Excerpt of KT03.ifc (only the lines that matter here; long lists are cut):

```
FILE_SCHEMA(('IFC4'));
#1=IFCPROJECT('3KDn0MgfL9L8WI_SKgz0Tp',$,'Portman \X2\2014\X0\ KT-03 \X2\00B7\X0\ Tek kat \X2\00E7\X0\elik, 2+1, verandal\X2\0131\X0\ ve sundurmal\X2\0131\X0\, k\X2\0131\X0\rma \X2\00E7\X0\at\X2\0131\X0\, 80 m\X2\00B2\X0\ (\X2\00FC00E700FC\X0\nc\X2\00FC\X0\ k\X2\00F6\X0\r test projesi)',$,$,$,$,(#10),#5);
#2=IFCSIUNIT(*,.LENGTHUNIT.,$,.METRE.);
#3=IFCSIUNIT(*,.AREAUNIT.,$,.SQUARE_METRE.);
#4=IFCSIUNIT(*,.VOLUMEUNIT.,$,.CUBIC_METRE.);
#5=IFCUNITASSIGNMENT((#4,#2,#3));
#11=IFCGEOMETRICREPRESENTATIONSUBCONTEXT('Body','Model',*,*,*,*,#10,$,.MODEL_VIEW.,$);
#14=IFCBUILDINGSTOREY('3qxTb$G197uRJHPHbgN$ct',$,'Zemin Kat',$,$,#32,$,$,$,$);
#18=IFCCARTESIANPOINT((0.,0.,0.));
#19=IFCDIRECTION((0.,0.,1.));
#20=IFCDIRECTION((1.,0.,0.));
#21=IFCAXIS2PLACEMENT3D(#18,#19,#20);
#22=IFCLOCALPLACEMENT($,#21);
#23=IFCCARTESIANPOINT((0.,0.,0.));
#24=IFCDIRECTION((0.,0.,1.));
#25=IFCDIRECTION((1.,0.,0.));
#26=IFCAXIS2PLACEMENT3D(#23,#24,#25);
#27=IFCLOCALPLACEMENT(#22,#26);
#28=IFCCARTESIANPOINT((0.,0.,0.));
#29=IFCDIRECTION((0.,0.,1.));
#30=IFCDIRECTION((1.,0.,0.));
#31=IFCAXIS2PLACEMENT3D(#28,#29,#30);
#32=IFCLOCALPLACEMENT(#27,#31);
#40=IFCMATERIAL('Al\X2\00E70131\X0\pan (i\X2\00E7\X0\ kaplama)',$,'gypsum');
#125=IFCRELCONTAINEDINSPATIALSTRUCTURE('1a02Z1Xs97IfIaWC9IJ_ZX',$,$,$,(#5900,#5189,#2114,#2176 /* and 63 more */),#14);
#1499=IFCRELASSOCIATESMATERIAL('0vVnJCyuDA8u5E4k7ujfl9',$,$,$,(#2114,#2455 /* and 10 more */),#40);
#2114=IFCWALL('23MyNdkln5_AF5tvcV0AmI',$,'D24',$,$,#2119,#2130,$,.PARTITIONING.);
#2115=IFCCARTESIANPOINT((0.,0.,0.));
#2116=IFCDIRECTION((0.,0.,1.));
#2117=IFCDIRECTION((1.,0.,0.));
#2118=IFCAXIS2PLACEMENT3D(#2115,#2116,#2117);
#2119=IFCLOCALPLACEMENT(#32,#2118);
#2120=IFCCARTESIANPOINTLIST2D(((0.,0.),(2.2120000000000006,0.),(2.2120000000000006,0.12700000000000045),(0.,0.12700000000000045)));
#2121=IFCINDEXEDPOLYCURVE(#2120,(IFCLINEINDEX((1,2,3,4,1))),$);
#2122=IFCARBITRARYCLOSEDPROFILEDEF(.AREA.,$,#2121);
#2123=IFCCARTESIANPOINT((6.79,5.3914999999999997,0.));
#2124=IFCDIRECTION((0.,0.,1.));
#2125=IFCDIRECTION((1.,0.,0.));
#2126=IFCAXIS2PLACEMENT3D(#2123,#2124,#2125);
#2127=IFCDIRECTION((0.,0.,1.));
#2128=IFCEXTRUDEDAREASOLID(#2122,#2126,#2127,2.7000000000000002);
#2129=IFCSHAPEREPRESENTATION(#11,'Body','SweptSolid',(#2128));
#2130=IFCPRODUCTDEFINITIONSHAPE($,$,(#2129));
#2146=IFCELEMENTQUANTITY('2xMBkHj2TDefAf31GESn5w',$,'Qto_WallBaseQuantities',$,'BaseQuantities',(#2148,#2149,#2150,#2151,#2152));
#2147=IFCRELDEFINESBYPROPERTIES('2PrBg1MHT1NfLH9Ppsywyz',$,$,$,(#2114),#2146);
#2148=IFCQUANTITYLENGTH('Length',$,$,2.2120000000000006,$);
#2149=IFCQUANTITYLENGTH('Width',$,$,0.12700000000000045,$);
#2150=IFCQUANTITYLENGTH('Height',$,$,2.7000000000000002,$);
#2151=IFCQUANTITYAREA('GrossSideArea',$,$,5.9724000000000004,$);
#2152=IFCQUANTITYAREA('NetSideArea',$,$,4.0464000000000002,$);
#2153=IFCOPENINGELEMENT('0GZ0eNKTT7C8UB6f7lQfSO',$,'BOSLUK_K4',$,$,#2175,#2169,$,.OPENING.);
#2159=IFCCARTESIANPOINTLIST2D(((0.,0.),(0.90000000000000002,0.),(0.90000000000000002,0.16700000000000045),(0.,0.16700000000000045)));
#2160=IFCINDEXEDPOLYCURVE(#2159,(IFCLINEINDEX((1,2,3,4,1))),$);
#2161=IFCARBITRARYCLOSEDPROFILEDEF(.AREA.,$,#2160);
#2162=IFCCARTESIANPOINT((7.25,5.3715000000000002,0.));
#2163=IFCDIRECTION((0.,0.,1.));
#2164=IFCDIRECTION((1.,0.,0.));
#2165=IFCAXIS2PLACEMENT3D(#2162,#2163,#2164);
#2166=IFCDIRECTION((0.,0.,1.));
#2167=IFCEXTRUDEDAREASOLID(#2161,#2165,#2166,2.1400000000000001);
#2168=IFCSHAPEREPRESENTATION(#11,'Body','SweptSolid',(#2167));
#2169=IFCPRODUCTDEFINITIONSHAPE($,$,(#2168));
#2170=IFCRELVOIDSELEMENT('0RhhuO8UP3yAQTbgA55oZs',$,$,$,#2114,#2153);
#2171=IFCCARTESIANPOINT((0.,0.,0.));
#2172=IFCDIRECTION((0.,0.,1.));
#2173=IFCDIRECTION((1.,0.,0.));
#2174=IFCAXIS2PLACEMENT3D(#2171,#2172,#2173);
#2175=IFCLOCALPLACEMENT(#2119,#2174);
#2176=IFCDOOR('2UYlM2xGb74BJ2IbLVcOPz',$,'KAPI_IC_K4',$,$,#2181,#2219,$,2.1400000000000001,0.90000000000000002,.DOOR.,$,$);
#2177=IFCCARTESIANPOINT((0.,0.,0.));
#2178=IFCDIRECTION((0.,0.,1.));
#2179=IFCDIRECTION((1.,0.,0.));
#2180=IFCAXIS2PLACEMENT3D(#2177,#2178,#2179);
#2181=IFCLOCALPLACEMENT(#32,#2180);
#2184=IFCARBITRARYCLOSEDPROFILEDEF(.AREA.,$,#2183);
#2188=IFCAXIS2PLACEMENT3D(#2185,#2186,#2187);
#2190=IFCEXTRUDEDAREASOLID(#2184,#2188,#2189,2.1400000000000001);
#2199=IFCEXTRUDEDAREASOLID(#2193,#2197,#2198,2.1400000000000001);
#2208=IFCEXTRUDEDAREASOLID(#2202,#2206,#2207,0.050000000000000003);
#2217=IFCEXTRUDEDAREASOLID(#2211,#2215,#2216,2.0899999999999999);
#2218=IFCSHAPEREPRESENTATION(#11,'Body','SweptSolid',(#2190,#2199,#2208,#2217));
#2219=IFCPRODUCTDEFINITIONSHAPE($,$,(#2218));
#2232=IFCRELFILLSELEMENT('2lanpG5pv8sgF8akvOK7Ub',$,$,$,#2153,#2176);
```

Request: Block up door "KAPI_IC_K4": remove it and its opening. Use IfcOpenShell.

```python
import ifcopenshell
import ifcopenshell.api.feature
import ifcopenshell.api.pset
import ifcopenshell.api.root
import ifcopenshell.geom
import ifcopenshell.util.element
import ifcopenshell.util.shape
import ifcopenshell.util.unit

model = ifcopenshell.open("KT03.ifc")
area_scale = ifcopenshell.util.unit.calculate_unit_scale(model, "AREAUNIT")
settings = ifcopenshell.geom.settings()


def volume(element):
    """Net volume in cubic metres, openings subtracted."""
    shape = ifcopenshell.geom.create_shape(settings, element)
    return ifcopenshell.util.shape.get_volume(shape.geometry)


door = model.by_guid("2UYlM2xGb74BJ2IbLVcOPz")
opening = door.FillsVoids[0].RelatingOpeningElement
wall = opening.VoidsElements[0].RelatingBuildingElement
before = volume(wall)

ifcopenshell.api.root.remove_product(model, product=door)
ifcopenshell.api.feature.remove_feature(model, feature=opening)

after = volume(wall)
thickness = 0.127  # wall thickness in metres

# Update the wall's stored quantities.
qto = model.by_id(ifcopenshell.util.element.get_pset(wall, "Qto_WallBaseQuantities", should_inherit=False)["id"])
ifcopenshell.api.pset.edit_qto(model, qto=qto, properties={"NetSideArea": after / thickness / area_scale})

print(f"wall volume {before:.3f} -> {after:.3f} m3")

model.write("KT03_rev.ifc")
```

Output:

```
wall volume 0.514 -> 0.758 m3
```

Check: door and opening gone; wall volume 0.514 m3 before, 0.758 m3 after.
